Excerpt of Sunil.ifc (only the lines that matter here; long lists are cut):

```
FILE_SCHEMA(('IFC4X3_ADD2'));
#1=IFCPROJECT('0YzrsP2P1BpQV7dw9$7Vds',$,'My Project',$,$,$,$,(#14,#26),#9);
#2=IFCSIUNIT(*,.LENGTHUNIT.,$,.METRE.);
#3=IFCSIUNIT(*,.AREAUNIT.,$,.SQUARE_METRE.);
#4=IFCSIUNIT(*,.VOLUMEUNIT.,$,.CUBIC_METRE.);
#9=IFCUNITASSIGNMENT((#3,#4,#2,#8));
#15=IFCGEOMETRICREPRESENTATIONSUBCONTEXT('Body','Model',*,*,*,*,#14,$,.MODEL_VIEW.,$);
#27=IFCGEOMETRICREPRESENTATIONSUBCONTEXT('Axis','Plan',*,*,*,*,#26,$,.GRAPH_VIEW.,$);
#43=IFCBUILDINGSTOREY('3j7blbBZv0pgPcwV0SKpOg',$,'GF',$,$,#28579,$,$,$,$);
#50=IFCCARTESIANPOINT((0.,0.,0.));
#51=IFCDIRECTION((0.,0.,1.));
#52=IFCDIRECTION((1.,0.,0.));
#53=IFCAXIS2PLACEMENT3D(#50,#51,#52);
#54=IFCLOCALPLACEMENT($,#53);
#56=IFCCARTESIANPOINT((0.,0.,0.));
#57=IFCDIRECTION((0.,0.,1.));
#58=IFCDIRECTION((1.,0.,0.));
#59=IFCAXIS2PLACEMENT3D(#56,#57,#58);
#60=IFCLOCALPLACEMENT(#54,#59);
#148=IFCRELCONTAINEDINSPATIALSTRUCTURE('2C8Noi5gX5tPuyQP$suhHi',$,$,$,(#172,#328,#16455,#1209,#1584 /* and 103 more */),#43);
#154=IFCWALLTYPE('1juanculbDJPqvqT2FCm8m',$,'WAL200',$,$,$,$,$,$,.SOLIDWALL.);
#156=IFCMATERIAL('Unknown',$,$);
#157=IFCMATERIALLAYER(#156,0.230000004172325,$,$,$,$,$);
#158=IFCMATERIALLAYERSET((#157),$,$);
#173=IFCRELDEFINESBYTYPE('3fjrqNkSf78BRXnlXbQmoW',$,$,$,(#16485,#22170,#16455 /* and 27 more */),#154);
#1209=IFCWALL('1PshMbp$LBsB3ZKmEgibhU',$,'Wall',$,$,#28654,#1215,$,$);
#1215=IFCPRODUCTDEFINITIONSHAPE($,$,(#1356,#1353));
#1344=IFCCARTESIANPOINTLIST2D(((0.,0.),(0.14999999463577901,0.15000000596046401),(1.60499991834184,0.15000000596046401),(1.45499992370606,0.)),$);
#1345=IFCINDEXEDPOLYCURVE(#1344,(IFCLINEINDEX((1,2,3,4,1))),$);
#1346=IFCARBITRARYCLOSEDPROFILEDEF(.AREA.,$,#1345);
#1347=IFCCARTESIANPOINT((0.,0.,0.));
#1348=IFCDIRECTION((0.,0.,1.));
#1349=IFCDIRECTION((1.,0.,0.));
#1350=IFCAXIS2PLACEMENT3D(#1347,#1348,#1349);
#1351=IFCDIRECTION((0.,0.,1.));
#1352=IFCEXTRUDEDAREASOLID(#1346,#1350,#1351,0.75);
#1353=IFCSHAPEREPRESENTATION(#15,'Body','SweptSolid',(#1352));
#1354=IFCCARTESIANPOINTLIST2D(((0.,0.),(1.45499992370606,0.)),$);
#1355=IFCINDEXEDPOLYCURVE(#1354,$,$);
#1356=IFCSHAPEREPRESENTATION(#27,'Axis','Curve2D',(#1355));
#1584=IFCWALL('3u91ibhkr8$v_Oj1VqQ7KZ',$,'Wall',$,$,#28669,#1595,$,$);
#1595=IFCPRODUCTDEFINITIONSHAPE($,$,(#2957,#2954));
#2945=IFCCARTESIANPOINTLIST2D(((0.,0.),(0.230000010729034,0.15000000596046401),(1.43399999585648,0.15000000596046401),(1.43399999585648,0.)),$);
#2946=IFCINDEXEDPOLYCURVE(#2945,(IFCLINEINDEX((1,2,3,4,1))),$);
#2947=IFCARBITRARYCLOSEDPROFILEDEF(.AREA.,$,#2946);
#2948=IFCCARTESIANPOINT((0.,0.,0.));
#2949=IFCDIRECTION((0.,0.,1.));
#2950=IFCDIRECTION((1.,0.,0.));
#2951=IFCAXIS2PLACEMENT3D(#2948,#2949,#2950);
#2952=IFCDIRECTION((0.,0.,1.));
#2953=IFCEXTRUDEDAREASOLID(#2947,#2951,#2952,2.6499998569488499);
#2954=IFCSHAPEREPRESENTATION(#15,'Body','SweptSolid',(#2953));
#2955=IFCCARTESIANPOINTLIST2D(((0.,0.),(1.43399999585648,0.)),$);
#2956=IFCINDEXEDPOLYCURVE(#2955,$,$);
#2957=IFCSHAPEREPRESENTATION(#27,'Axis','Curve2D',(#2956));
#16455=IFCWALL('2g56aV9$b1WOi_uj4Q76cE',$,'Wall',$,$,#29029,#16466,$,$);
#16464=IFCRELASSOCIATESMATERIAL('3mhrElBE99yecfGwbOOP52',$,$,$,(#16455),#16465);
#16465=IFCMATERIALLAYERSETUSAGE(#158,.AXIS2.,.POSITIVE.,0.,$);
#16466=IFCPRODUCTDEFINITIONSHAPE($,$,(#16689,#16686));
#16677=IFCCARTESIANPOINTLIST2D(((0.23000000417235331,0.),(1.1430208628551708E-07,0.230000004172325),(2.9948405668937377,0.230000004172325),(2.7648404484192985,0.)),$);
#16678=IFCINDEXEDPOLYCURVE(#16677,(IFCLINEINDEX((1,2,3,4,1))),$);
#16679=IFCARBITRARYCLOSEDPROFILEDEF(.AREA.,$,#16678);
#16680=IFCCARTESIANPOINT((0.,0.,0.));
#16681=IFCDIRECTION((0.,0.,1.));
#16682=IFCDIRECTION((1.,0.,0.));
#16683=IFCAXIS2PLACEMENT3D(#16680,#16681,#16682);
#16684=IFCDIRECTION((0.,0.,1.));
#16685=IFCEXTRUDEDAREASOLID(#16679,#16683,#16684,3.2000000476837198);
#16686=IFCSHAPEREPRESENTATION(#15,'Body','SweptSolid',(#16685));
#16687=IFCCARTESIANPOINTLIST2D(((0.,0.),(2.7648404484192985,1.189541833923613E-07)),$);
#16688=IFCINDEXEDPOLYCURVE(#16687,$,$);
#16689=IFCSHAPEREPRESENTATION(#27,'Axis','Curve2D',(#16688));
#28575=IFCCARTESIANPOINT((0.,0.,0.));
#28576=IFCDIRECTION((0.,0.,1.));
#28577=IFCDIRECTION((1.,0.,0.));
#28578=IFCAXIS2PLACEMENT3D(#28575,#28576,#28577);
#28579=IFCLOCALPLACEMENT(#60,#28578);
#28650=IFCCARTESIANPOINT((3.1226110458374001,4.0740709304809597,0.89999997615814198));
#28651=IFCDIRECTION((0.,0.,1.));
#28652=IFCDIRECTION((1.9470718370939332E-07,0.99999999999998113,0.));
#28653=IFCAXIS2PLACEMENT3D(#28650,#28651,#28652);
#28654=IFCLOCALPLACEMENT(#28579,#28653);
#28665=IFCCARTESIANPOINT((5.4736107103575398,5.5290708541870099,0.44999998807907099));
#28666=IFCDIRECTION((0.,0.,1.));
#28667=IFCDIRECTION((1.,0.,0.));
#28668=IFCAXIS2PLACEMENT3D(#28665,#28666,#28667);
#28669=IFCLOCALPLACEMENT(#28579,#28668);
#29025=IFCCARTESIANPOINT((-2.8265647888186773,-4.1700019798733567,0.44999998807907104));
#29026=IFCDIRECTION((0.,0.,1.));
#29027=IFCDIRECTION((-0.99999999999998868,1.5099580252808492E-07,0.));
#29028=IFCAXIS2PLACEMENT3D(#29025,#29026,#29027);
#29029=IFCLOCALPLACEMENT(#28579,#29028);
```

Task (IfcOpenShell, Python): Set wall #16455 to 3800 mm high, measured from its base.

```python
import ifcopenshell
import ifcopenshell.geom
import ifcopenshell.util.representation
import ifcopenshell.util.shape
import ifcopenshell.util.unit

model = ifcopenshell.open("Sunil.ifc")
unit_scale = ifcopenshell.util.unit.calculate_unit_scale(model)
settings = ifcopenshell.geom.settings()


def volume(element):
    """Net volume in cubic metres, openings subtracted."""
    shape = ifcopenshell.geom.create_shape(settings, element)
    return ifcopenshell.util.shape.get_volume(shape.geometry)


wall = model.by_guid("2g56aV9$b1WOi_uj4Q76cE")
before = volume(wall)

body = ifcopenshell.util.representation.get_representation(wall, "Model", "Body")
solid = body.Items[0]
old_height = solid.Depth
solid.Depth = 3.8 / unit_scale
after = volume(wall)

print(f"height {old_height:g} -> {solid.Depth:g}, volume {before:.3f} -> {after:.3f} m3")

model.write("Sunil_edited.ifc")
```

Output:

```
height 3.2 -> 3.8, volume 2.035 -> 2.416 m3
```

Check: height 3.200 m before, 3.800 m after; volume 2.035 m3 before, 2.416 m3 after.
